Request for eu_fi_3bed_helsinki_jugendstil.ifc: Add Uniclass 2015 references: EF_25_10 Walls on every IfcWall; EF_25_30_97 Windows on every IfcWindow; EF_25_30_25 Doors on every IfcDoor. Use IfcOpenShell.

First a look at what the model holds.

```python
import ifcopenshell

model = ifcopenshell.open("eu_fi_3bed_helsinki_jugendstil.ifc")
print(model.schema)
print("classifications:", [c.Name for c in model.by_type("IfcClassification")])
for ifc_class in ("IfcDoor", "IfcRoof", "IfcStair", "IfcWall", "IfcWindow"):
    print(ifc_class, len(model.by_type(ifc_class)))
```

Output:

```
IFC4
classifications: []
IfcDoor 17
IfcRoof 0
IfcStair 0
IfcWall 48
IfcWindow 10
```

```python
import ifcopenshell
import ifcopenshell.api.classification

model = ifcopenshell.open("eu_fi_3bed_helsinki_jugendstil.ifc")

system = ifcopenshell.api.classification.add_classification(model, classification="Uniclass 2015")

codes = {
    "IfcWall": ("EF_25_10", "Walls"),
    "IfcWindow": ("EF_25_30_97", "Windows"),
    "IfcDoor": ("EF_25_30_25", "Doors"),
}
for ifc_class, (code, name) in codes.items():
    products = model.by_type(ifc_class)
    ifcopenshell.api.classification.add_reference(
        model, products=products, classification=system, identification=code, name=name
    )
    print(code, len(products))

model.write("eu_fi_3bed_helsinki_jugendstil-out.ifc")
```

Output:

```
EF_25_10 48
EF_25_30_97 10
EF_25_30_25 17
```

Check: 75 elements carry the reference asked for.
